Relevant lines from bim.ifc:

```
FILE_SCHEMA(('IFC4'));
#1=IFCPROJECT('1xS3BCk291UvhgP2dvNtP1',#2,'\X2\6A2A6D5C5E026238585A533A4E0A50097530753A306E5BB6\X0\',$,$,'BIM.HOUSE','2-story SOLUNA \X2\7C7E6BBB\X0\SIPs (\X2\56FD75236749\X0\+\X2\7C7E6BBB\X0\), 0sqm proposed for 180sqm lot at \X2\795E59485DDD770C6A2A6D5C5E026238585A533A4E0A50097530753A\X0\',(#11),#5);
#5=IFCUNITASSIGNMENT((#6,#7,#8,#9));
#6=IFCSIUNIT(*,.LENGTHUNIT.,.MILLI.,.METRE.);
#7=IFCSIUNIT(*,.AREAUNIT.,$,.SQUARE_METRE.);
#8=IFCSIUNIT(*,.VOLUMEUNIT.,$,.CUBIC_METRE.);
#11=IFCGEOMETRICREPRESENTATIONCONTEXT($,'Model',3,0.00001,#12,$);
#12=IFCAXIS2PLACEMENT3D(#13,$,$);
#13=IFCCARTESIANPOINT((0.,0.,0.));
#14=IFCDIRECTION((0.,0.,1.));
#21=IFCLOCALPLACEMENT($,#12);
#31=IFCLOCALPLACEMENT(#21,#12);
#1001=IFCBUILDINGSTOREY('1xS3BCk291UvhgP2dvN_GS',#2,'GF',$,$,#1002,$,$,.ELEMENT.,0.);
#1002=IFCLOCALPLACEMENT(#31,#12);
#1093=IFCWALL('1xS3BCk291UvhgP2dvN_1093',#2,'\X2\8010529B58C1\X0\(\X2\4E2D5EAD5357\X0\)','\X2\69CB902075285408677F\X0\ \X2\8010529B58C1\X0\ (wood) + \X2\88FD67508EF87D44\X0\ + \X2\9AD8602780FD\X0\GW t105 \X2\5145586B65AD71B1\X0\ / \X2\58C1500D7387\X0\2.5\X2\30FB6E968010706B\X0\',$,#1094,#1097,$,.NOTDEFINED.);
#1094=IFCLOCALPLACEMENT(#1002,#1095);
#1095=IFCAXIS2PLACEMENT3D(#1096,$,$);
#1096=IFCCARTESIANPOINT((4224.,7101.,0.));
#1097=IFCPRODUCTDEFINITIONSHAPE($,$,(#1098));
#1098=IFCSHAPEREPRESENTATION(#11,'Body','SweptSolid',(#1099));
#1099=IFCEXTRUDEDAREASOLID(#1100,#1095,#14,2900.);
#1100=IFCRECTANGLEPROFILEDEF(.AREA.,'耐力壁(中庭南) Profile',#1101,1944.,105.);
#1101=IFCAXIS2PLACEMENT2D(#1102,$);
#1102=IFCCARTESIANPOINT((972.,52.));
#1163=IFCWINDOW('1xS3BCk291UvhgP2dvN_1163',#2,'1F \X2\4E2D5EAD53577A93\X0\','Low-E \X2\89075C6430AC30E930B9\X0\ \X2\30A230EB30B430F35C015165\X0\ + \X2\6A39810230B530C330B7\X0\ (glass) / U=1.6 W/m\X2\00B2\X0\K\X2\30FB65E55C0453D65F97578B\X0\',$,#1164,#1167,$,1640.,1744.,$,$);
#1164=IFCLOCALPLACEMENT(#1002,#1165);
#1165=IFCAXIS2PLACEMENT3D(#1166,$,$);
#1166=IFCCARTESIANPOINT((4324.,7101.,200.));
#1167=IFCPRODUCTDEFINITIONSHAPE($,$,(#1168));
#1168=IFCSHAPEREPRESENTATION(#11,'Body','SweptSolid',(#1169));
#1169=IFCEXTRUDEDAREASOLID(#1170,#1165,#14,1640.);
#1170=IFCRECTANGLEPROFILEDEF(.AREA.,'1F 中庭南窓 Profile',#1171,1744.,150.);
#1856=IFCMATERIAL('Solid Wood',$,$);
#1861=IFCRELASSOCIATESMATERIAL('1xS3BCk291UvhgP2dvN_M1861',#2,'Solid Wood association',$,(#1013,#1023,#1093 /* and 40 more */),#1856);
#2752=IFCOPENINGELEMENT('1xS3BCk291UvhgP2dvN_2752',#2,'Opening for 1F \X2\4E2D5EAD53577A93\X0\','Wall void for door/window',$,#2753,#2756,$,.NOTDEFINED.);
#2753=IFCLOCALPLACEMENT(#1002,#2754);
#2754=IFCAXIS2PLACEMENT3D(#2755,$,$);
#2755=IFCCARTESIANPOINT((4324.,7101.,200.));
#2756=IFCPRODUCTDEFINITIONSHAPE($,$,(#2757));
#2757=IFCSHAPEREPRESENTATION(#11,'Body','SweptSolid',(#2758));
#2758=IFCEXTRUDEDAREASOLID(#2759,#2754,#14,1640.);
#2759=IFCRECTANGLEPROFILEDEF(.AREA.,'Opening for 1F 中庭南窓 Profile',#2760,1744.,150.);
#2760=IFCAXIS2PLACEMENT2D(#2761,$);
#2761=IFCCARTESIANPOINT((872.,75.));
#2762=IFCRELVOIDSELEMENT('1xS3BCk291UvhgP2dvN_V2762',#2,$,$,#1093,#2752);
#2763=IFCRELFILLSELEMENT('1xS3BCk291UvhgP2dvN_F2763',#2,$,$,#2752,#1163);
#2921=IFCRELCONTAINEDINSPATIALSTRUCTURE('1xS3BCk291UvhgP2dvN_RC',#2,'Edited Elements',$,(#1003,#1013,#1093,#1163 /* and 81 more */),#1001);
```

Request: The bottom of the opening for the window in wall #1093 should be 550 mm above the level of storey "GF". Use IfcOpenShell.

```python
import numpy as np
import ifcopenshell
import ifcopenshell.api.geometry
import ifcopenshell.geom
import ifcopenshell.util.element
import ifcopenshell.util.placement
import ifcopenshell.util.shape
import ifcopenshell.util.unit

model = ifcopenshell.open("bim.ifc")
unit_scale = ifcopenshell.util.unit.calculate_unit_scale(model)

window = model.by_guid("1xS3BCk291UvhgP2dvN_1163")
opening = window.FillsVoids[0].RelatingOpeningElement
storey = ifcopenshell.util.element.get_container(window, ifc_class="IfcBuildingStorey")
level = ifcopenshell.util.placement.get_local_placement(storey.ObjectPlacement)[2, 3]

# The opening's origin need not be at the sill, so measure its lowest point.
shape = ifcopenshell.geom.create_shape(ifcopenshell.geom.settings(), opening)
bottom = ifcopenshell.util.shape.get_shape_bottom_elevation(shape, shape.geometry) / unit_scale
dz = level + 0.55 / unit_scale - bottom

shift = np.array([0.0, 0.0, dz])
# The window is not placed relative to its opening, so move both.
for product in (opening, window):
    matrix = ifcopenshell.util.placement.get_local_placement(product.ObjectPlacement)
    matrix[:3, 3] += shift
    ifcopenshell.api.geometry.edit_object_placement(model, product=product, matrix=matrix, is_si=False)

print(f"moved by {dz * unit_scale:+.3f} m")

model.write("bim_edited.ifc")
```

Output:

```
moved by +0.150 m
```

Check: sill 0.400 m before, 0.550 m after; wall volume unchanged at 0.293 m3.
